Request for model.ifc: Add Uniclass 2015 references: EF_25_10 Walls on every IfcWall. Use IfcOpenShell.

First a look at what the model holds.

```python
import ifcopenshell

model = ifcopenshell.open("model.ifc")
print(model.schema)
print("classifications:", [c.Name for c in model.by_type("IfcClassification")])
for ifc_class in ("IfcDoor", "IfcRoof", "IfcStair", "IfcWall", "IfcWindow"):
    print(ifc_class, len(model.by_type(ifc_class)))
```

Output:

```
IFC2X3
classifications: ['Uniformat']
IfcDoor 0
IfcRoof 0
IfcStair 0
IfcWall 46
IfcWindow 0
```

```python
import ifcopenshell
import ifcopenshell.api.classification

model = ifcopenshell.open("model.ifc")

# IFC2X3 requires Source and Edition and has no link from the project to the system.
system = model.create_entity("IfcClassification", Source="NBS", Edition="2015", Name="Uniclass 2015")

codes = {
    "IfcWall": ("EF_25_10", "Walls"),
}
for ifc_class, (code, name) in codes.items():
    products = model.by_type(ifc_class)
    ifcopenshell.api.classification.add_reference(
        model, products=products, classification=system, identification=code, name=name
    )
    print(code, len(products))

model.write("model_v2.ifc")
```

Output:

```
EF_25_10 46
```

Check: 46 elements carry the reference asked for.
